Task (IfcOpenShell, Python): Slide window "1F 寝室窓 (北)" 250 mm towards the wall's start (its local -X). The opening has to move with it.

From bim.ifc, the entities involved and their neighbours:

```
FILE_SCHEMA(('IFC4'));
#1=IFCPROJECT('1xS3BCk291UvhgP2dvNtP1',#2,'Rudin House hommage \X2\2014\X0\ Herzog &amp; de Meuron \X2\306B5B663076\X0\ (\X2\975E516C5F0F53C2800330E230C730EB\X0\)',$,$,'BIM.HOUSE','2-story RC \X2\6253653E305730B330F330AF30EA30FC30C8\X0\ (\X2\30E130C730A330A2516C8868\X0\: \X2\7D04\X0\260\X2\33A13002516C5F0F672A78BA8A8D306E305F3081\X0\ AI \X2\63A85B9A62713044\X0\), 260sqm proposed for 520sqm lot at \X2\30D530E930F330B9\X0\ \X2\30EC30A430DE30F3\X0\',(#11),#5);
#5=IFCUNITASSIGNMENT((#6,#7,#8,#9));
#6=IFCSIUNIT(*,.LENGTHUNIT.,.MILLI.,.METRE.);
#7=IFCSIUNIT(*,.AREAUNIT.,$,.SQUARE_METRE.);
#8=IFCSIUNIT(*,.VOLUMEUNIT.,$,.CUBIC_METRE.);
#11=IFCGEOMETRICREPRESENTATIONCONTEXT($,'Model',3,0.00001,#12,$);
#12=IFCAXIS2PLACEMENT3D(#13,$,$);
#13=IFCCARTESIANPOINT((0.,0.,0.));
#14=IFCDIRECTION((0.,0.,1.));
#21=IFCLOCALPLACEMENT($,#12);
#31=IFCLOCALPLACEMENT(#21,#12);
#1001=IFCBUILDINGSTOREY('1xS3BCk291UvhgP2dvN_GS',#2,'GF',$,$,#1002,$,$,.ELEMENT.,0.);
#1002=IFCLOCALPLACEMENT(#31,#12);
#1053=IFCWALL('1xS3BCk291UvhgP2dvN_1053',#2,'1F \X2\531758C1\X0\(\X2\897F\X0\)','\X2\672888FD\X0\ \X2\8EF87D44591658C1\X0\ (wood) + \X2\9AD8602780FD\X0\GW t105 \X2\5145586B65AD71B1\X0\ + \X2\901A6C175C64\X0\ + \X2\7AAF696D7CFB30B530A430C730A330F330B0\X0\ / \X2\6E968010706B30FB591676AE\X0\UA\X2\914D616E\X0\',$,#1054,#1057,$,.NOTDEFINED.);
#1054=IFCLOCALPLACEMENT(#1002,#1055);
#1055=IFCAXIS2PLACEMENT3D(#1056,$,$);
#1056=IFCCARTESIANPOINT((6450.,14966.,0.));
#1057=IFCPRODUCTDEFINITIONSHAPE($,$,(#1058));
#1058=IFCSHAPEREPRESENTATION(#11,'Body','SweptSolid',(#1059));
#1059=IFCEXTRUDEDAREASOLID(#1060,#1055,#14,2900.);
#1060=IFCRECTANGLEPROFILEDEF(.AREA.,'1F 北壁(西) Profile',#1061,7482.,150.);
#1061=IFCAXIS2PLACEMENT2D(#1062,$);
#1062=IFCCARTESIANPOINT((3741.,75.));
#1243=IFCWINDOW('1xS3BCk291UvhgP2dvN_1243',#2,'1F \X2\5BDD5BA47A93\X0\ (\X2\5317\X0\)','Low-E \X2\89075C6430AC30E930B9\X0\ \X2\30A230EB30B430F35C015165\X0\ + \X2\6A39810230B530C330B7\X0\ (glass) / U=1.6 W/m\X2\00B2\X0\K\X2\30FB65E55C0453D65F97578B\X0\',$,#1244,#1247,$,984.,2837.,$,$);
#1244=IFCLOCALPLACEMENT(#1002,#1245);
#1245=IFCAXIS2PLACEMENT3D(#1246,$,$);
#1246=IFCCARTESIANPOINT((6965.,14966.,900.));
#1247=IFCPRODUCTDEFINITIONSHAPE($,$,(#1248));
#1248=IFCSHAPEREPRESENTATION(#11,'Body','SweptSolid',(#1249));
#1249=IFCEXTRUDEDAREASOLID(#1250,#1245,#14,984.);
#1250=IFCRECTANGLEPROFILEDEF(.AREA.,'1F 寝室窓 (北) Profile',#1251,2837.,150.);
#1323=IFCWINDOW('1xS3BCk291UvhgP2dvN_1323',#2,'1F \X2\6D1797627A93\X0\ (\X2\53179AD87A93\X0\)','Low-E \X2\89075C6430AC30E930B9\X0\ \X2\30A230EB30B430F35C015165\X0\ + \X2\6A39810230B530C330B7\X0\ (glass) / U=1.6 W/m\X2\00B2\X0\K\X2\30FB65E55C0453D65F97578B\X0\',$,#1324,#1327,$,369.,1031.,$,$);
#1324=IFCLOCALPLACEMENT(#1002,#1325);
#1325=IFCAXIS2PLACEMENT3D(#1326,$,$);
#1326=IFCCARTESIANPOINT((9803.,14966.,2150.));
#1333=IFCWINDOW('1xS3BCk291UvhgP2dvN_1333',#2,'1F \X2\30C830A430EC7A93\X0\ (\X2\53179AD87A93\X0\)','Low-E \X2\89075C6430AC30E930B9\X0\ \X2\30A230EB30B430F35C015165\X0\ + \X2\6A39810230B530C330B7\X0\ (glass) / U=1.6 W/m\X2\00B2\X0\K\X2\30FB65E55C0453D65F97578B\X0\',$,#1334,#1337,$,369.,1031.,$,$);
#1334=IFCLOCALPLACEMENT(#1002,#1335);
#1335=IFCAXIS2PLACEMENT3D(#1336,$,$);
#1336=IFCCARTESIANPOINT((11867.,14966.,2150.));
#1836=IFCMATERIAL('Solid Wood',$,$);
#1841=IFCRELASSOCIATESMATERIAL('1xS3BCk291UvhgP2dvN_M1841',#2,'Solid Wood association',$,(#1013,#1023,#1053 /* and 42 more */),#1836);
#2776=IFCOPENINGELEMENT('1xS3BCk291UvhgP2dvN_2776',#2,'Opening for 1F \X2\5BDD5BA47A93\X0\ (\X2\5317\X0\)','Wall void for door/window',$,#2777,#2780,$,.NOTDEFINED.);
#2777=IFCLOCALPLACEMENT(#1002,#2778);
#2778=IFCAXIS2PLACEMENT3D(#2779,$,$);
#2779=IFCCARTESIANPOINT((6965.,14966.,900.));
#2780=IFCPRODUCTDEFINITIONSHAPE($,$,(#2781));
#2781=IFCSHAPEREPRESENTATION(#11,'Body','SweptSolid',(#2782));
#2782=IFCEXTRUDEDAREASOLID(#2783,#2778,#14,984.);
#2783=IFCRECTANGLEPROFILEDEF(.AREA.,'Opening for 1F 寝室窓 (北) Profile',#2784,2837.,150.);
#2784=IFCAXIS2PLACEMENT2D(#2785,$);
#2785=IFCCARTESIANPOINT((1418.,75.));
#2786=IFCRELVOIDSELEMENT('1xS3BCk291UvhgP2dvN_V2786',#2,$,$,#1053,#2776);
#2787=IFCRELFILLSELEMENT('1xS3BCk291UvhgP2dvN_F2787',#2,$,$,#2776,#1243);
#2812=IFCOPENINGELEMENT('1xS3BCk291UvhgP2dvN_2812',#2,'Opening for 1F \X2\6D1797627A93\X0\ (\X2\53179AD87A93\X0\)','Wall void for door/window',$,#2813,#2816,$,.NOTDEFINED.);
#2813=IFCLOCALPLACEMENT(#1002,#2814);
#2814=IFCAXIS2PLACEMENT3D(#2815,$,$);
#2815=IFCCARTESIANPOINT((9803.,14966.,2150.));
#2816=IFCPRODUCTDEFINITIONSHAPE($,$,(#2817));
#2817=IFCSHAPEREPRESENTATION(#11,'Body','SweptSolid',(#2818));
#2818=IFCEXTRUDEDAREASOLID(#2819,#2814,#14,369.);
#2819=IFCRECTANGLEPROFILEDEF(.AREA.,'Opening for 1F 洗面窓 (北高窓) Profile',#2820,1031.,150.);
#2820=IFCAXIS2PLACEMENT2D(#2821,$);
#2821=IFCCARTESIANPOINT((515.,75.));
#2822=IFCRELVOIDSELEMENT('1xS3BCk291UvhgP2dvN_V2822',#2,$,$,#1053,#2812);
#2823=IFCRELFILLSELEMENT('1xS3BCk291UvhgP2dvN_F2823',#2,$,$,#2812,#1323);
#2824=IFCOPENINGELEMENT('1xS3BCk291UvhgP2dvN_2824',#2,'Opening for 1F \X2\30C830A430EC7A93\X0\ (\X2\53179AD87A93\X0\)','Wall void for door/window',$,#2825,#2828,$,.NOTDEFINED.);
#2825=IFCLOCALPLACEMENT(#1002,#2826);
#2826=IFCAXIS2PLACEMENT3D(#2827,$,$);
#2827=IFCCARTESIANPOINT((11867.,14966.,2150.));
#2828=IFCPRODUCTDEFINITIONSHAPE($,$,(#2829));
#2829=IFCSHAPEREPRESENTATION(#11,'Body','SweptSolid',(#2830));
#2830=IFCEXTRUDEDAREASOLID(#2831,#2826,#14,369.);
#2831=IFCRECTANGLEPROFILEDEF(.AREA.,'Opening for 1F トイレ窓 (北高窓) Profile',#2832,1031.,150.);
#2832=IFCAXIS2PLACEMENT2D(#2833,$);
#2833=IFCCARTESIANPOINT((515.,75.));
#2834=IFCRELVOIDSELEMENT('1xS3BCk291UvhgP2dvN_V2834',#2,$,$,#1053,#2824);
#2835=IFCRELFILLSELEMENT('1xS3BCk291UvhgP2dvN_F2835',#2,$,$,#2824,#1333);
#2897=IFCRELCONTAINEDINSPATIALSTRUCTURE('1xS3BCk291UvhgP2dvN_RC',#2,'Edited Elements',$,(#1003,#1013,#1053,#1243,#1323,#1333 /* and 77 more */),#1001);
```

```python
import ifcopenshell
import ifcopenshell.api.geometry
import ifcopenshell.util.placement

model = ifcopenshell.open("bim.ifc")

window = model.by_guid("1xS3BCk291UvhgP2dvN_1243")
opening = window.FillsVoids[0].RelatingOpeningElement
wall = opening.VoidsElements[0].RelatingBuildingElement

wall_matrix = ifcopenshell.util.placement.get_local_placement(wall.ObjectPlacement)
shift = wall_matrix[:3, 0] * -250.0
before = ifcopenshell.util.placement.get_local_placement(window.ObjectPlacement)[:3, 3].copy()

# The window is not placed relative to its opening, so move both.
for product in (opening, window):
    matrix = ifcopenshell.util.placement.get_local_placement(product.ObjectPlacement)
    matrix[:3, 3] += shift
    ifcopenshell.api.geometry.edit_object_placement(model, product=product, matrix=matrix, is_si=False)

after = ifcopenshell.util.placement.get_local_placement(window.ObjectPlacement)[:3, 3]
print("window moved by", (after - before).round(3) + 0.0)

model.write("bim_rev.ifc")
```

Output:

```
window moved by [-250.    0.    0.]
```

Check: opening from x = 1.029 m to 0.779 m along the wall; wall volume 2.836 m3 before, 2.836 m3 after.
